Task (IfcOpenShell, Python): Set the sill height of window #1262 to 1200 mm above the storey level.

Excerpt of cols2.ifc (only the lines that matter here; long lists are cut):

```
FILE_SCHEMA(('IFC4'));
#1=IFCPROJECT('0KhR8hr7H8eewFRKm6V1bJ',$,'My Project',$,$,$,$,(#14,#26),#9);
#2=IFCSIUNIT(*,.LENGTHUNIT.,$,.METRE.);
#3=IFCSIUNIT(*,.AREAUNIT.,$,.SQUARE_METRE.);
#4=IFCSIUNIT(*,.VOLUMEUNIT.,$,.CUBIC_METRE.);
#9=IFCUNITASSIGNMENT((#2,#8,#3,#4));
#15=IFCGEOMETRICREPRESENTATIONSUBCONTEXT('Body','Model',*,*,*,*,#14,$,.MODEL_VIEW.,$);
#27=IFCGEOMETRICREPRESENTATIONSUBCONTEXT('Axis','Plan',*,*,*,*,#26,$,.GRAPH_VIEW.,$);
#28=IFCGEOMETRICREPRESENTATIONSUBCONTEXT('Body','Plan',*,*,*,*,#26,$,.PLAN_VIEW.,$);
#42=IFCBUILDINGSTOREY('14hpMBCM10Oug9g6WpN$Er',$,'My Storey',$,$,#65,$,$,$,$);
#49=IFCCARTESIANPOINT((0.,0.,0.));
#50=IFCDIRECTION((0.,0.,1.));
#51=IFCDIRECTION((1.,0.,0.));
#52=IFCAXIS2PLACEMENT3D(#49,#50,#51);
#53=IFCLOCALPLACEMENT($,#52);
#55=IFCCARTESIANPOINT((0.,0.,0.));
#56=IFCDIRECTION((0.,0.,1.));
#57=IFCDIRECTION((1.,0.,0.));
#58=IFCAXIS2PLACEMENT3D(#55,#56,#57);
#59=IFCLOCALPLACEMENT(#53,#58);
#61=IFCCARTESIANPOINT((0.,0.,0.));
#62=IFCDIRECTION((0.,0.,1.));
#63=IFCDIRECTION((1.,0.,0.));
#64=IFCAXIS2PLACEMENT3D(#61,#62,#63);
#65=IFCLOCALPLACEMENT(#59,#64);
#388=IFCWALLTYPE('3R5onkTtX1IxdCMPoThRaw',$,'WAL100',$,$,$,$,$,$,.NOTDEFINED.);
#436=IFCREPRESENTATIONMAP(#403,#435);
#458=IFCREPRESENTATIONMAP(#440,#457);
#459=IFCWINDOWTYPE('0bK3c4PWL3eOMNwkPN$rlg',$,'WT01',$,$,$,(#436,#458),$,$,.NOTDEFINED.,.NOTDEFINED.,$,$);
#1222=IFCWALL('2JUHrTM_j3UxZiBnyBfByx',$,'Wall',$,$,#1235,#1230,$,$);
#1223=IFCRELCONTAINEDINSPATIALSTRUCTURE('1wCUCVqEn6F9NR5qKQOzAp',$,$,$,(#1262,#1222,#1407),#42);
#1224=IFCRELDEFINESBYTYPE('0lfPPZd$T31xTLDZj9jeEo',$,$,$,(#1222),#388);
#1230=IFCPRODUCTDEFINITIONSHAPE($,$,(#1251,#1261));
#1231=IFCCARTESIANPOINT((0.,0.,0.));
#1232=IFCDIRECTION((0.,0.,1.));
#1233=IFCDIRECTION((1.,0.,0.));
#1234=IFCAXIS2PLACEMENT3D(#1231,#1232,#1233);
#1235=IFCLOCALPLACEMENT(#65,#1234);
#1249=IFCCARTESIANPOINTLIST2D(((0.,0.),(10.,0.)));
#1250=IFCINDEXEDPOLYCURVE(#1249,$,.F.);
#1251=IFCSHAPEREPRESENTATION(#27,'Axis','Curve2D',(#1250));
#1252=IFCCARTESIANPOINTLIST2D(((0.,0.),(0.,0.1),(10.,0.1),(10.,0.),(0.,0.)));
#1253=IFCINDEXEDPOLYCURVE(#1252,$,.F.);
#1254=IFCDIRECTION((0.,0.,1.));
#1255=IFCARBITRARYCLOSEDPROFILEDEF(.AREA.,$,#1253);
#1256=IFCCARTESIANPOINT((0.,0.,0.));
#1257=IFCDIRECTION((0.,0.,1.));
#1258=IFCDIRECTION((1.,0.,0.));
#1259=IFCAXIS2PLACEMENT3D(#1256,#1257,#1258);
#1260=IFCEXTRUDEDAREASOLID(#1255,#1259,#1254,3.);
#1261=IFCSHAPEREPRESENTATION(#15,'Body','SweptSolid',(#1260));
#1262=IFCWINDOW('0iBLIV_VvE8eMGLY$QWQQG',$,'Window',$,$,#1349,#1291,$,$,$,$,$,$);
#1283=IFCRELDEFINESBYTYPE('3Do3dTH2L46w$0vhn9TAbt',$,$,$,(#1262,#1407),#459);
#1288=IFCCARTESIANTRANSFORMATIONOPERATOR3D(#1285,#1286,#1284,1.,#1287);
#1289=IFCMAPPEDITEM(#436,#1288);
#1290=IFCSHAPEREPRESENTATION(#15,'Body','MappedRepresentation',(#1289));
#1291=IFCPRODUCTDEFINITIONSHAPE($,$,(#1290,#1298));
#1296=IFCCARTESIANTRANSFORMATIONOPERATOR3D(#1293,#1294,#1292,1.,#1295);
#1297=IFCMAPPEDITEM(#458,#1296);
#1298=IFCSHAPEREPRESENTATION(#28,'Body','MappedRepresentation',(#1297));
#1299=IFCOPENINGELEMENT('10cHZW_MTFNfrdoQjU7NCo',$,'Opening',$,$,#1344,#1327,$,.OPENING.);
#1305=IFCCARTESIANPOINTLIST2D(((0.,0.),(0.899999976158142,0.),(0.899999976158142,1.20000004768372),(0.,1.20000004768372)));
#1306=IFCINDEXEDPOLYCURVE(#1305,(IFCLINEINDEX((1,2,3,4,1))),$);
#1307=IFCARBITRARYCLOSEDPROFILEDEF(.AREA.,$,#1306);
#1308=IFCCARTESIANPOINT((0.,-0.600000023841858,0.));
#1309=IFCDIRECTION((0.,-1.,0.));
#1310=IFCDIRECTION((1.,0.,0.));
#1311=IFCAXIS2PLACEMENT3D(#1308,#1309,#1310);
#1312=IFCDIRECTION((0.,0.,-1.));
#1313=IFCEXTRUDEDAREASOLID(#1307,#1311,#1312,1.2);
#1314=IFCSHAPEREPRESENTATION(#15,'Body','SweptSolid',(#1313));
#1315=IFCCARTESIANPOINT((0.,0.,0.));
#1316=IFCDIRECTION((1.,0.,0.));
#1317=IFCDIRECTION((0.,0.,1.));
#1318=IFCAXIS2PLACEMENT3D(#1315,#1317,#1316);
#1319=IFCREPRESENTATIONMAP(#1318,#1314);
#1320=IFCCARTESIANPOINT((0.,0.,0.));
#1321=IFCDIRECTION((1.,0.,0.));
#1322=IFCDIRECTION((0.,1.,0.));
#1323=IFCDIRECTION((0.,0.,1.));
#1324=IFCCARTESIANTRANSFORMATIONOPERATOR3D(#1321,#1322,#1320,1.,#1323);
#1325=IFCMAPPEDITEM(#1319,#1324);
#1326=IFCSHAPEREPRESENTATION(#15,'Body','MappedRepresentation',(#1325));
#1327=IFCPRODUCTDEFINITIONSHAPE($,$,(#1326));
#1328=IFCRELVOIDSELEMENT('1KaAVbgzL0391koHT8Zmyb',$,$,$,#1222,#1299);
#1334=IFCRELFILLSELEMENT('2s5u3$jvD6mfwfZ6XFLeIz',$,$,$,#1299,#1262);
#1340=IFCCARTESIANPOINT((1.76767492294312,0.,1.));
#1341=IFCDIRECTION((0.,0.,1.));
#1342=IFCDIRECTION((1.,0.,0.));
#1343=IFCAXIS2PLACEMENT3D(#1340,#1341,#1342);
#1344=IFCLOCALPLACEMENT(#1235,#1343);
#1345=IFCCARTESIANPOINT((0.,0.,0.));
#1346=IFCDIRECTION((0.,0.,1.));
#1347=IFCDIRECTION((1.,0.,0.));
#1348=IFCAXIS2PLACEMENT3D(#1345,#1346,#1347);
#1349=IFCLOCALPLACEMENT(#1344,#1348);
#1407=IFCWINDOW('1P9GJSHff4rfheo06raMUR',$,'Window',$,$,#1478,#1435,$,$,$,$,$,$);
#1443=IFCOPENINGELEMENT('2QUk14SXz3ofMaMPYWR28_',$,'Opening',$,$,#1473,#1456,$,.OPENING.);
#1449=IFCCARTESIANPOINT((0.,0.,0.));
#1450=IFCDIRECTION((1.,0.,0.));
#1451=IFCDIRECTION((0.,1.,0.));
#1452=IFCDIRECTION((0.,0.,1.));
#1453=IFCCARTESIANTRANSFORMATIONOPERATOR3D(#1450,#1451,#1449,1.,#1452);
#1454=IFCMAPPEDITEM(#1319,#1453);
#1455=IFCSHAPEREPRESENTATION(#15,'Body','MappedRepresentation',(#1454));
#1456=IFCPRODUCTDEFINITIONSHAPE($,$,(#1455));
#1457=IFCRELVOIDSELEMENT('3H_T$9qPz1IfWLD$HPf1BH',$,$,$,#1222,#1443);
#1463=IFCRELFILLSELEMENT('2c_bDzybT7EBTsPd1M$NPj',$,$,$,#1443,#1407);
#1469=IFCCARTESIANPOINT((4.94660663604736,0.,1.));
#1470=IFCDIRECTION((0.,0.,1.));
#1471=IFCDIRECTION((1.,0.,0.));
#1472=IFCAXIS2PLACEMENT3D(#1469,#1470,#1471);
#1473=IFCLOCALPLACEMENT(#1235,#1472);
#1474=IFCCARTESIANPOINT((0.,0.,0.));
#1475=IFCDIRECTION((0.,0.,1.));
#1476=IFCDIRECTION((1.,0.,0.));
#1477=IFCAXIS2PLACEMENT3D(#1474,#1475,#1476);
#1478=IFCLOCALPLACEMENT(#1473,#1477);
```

```python
import numpy as np
import ifcopenshell
import ifcopenshell.api.geometry
import ifcopenshell.geom
import ifcopenshell.util.element
import ifcopenshell.util.placement
import ifcopenshell.util.shape
import ifcopenshell.util.unit

model = ifcopenshell.open("cols2.ifc")
unit_scale = ifcopenshell.util.unit.calculate_unit_scale(model)

window = model.by_guid("0iBLIV_VvE8eMGLY$QWQQG")
opening = window.FillsVoids[0].RelatingOpeningElement
storey = ifcopenshell.util.element.get_container(window, ifc_class="IfcBuildingStorey")
level = ifcopenshell.util.placement.get_local_placement(storey.ObjectPlacement)[2, 3]

# The opening's origin need not be at the sill, so measure its lowest point.
shape = ifcopenshell.geom.create_shape(ifcopenshell.geom.settings(), opening)
bottom = ifcopenshell.util.shape.get_shape_bottom_elevation(shape, shape.geometry) / unit_scale
dz = level + 1.2 - bottom

shift = np.array([0.0, 0.0, dz])
# The window is placed relative to its opening, so it follows when the opening moves.
matrix = ifcopenshell.util.placement.get_local_placement(opening.ObjectPlacement)
matrix[:3, 3] += shift
ifcopenshell.api.geometry.edit_object_placement(
    model, product=opening, matrix=matrix, is_si=False, should_transform_children=True
)

print(f"moved by {dz * unit_scale:+.3f} m")

model.write("cols2_rev.ifc")
```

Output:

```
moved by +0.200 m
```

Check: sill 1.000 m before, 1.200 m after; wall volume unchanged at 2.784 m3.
